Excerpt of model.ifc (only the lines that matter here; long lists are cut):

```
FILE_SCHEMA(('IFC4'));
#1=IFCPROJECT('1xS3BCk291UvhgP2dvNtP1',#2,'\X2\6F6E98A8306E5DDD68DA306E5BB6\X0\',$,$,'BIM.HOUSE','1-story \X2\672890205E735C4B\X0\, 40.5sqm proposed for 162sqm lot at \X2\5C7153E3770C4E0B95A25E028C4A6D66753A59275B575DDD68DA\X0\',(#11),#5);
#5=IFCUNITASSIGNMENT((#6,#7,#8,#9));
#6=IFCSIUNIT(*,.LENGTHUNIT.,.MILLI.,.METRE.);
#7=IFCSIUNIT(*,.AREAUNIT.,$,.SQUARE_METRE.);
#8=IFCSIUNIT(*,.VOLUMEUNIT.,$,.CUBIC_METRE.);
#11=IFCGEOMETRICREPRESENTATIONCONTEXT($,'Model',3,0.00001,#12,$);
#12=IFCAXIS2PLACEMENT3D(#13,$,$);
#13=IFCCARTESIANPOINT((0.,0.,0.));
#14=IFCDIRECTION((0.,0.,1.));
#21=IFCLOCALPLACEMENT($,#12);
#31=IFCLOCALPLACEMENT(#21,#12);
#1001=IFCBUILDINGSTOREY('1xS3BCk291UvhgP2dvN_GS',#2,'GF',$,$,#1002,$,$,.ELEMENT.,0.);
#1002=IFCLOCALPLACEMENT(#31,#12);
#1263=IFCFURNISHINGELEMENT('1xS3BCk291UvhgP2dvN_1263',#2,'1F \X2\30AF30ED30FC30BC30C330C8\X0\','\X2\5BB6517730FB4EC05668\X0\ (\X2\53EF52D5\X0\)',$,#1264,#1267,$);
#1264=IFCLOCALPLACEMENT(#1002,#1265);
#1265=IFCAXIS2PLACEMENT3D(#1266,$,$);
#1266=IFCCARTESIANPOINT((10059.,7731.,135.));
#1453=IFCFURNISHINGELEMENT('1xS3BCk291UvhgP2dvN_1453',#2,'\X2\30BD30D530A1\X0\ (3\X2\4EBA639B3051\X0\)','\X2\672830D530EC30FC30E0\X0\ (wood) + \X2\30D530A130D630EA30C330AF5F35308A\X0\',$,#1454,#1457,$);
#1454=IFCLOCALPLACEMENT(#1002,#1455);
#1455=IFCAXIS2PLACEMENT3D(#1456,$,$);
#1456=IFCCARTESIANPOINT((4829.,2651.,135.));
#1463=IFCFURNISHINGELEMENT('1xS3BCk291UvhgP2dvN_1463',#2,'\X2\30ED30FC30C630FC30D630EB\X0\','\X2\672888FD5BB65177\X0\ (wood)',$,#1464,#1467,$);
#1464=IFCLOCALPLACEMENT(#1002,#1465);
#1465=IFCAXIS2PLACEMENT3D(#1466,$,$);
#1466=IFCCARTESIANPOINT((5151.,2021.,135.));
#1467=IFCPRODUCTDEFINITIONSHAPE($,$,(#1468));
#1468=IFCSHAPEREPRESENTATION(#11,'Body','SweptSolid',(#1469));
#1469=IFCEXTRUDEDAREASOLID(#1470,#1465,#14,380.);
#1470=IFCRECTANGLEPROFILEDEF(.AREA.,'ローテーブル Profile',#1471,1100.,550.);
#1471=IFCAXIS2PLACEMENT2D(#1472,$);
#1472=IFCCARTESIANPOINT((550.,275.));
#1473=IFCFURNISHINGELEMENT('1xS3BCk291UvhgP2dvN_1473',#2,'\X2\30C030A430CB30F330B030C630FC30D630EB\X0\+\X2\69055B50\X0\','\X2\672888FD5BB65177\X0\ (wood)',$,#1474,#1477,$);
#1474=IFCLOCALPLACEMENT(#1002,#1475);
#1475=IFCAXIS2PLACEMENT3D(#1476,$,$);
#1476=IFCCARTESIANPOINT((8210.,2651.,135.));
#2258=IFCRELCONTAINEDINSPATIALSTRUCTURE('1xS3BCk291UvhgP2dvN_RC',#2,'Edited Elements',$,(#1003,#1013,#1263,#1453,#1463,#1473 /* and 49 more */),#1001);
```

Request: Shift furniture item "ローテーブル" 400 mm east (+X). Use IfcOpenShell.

```python
import ifcopenshell
import ifcopenshell.api.geometry
import ifcopenshell.util.placement

model = ifcopenshell.open("model.ifc")

item = model.by_guid("1xS3BCk291UvhgP2dvN_1463")
matrix = ifcopenshell.util.placement.get_local_placement(item.ObjectPlacement)
matrix[0, 3] += 400.0
ifcopenshell.api.geometry.edit_object_placement(model, product=item, matrix=matrix, is_si=False)

print(ifcopenshell.util.placement.get_local_placement(item.ObjectPlacement).round(3) + 0.0)

model.write("model_rev.ifc")
```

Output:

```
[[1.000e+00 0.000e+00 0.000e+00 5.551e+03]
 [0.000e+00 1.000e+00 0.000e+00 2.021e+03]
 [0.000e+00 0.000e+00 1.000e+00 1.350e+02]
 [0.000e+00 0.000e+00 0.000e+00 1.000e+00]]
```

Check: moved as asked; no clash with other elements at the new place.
